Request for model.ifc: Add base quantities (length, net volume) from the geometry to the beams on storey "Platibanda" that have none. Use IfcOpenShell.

First a look at what the model holds.

```python
import ifcopenshell
import ifcopenshell.util.element
import ifcopenshell.util.unit

model = ifcopenshell.open("model.ifc")
print(model.schema)
for unit_type in ("LENGTHUNIT", "AREAUNIT", "VOLUMEUNIT"):
    print(unit_type, ifcopenshell.util.unit.calculate_unit_scale(model, unit_type))
storey = next(s for s in model.by_type("IfcBuildingStorey") if s.Name == "Platibanda")
beams = [e for e in ifcopenshell.util.element.get_decomposition(storey) if e.is_a("IfcBeam")]
for e in sorted(beams, key=lambda e: e.id()):
    print(e.id(), e.is_a(), e.Name, list(ifcopenshell.util.element.get_psets(e, qtos_only=True)), sep=" | ")
```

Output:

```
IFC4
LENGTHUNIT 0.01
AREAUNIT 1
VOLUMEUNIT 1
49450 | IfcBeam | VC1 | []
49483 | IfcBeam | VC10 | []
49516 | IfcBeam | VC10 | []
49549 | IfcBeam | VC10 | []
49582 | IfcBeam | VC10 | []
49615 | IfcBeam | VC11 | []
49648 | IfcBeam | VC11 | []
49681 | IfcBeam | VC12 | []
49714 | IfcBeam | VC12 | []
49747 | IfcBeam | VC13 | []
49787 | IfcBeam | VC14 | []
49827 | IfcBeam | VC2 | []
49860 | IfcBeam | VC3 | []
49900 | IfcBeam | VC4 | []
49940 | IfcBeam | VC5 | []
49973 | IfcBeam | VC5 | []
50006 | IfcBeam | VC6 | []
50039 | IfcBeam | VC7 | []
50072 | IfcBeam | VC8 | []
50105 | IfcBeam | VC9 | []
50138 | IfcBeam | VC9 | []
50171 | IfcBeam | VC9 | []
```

```python
import ifcopenshell
import ifcopenshell.api.pset
import ifcopenshell.geom
import ifcopenshell.util.element
import ifcopenshell.util.shape
import ifcopenshell.util.unit

model = ifcopenshell.open("model.ifc")
unit_scale = ifcopenshell.util.unit.calculate_unit_scale(model)
volume_scale = ifcopenshell.util.unit.calculate_unit_scale(model, "VOLUMEUNIT")
settings = ifcopenshell.geom.settings()

storey = next(s for s in model.by_type("IfcBuildingStorey") if s.Name == "Platibanda")
beams = [e for e in ifcopenshell.util.element.get_decomposition(storey) if e.is_a("IfcBeam")]

for e in sorted(beams, key=lambda e: e.id()):
    if ifcopenshell.util.element.get_psets(e, qtos_only=True, should_inherit=False):
        continue
    # Geometry comes back in metres, in the element's own axes.
    shape = ifcopenshell.geom.create_shape(settings, e)
    values = {
        "Length": ifcopenshell.util.shape.get_max_xyz(shape.geometry) / unit_scale,
        "NetVolume": ifcopenshell.util.shape.get_volume(shape.geometry) / volume_scale,
    }
    qto = ifcopenshell.api.pset.add_qto(model, product=e, name="Qto_BeamBaseQuantities")
    ifcopenshell.api.pset.edit_qto(model, qto=qto, properties=values)
    print(e.id(), {k: round(v, 3) for k, v in values.items()})

model.write("model-out.ifc")
```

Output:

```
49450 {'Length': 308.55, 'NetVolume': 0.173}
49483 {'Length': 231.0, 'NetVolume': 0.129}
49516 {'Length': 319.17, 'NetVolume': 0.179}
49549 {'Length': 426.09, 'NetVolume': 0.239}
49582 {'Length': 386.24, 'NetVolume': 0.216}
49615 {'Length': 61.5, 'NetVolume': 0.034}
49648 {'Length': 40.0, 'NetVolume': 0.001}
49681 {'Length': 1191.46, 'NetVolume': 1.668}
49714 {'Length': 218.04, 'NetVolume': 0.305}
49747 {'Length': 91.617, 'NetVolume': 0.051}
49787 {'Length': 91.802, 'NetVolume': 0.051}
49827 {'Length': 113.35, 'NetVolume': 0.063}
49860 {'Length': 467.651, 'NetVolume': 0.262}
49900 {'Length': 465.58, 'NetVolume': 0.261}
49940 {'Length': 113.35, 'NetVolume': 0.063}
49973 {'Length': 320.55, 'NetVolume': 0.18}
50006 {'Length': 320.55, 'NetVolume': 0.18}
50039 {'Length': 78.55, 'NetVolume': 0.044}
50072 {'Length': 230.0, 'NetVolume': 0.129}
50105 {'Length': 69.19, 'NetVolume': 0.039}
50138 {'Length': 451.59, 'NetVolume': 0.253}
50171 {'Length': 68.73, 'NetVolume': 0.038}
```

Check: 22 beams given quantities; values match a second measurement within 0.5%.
